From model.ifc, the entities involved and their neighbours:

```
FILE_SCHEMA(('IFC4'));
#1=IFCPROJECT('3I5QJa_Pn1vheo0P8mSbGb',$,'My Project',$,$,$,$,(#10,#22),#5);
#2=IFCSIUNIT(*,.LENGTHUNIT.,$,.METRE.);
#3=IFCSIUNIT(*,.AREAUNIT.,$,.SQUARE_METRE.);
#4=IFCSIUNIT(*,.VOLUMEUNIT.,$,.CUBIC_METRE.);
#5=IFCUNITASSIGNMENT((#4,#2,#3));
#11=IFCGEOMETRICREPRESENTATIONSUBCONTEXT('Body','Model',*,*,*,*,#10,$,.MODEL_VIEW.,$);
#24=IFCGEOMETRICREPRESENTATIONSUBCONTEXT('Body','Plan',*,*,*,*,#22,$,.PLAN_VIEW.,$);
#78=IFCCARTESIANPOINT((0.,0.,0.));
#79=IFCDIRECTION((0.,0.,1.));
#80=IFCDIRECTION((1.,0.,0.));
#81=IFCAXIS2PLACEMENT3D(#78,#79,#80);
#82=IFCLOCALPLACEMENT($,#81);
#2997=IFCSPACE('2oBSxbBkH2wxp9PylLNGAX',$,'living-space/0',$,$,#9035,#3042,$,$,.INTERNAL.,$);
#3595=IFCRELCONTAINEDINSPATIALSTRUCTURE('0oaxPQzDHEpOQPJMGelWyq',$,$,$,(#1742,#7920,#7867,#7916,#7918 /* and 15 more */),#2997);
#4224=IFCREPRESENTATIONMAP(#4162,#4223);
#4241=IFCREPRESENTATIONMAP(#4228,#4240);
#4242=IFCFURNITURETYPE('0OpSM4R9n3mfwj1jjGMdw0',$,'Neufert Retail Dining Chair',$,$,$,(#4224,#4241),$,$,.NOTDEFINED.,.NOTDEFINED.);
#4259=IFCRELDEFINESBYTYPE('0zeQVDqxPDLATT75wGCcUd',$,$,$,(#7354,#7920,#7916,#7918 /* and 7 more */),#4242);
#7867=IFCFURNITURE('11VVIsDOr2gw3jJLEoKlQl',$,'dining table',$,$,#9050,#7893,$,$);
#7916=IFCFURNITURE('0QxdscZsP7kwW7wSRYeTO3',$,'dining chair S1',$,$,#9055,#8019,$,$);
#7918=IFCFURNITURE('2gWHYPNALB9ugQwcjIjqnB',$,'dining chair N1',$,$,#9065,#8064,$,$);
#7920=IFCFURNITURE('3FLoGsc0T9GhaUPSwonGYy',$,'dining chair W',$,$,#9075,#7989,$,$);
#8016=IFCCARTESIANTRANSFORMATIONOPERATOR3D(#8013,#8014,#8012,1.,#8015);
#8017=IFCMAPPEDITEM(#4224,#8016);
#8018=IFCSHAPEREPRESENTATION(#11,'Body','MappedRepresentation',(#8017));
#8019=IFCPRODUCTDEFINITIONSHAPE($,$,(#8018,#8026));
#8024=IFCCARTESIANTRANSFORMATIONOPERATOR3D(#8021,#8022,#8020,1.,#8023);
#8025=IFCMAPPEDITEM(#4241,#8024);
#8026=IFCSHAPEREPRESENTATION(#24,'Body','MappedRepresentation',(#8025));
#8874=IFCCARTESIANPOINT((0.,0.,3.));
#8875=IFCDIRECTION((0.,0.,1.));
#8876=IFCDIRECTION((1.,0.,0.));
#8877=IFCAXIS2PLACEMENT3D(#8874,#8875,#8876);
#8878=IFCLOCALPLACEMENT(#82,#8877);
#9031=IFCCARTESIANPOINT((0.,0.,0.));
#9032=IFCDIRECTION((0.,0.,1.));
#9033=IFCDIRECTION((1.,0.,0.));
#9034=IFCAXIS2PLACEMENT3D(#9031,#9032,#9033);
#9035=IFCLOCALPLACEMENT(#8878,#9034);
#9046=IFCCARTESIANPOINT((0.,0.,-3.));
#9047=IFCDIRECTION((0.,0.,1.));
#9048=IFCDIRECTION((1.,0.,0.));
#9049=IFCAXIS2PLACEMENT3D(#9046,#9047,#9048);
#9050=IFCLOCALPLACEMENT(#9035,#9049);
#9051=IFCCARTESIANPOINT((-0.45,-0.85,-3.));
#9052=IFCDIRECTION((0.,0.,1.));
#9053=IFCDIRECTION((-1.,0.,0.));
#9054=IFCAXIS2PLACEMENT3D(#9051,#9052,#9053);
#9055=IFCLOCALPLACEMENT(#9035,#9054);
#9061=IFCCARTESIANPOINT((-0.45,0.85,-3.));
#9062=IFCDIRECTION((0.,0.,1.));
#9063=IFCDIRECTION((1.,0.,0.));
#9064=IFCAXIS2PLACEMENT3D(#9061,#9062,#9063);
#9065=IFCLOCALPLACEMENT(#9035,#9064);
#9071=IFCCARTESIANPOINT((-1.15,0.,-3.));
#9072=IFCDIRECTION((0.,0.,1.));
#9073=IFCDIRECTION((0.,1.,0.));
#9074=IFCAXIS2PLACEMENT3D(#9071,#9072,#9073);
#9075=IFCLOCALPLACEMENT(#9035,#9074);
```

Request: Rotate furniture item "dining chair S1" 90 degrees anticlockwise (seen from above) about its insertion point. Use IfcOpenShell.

```python
import ifcopenshell
import ifcopenshell.api.geometry
import ifcopenshell.util.placement

model = ifcopenshell.open("model.ifc")

item = model.by_id(7916)
matrix = ifcopenshell.util.placement.get_local_placement(item.ObjectPlacement)
matrix = matrix @ ifcopenshell.util.placement.rotation(90, "Z")
ifcopenshell.api.geometry.edit_object_placement(model, product=item, matrix=matrix, is_si=False)

print(ifcopenshell.util.placement.get_local_placement(item.ObjectPlacement).round(3) + 0.0)

model.write("model_v2.ifc")
```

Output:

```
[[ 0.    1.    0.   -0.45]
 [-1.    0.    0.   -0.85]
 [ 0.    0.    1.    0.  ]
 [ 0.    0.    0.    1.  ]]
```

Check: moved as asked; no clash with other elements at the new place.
